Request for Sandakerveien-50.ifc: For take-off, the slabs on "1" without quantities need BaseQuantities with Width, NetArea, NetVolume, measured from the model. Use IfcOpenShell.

First a look at what the model holds.

```python
import ifcopenshell
import ifcopenshell.util.element
import ifcopenshell.util.unit

model = ifcopenshell.open("Sandakerveien-50.ifc")
print(model.schema)
for unit_type in ("LENGTHUNIT", "AREAUNIT", "VOLUMEUNIT"):
    print(unit_type, ifcopenshell.util.unit.calculate_unit_scale(model, unit_type))
storey = next(s for s in model.by_type("IfcBuildingStorey") if s.Name == "1")
slabs = [e for e in ifcopenshell.util.element.get_decomposition(storey) if e.is_a("IfcSlab")]
for e in sorted(slabs, key=lambda e: e.id()):
    print(e.id(), e.is_a(), e.Name, list(ifcopenshell.util.element.get_psets(e, qtos_only=True)), sep=" | ")
```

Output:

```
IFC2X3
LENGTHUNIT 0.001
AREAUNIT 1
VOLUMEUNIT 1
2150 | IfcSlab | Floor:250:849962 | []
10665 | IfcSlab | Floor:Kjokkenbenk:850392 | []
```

```python
import ifcopenshell
import ifcopenshell.api.pset
import ifcopenshell.geom
import ifcopenshell.util.element
import ifcopenshell.util.shape
import ifcopenshell.util.unit

model = ifcopenshell.open("Sandakerveien-50.ifc")
unit_scale = ifcopenshell.util.unit.calculate_unit_scale(model)
area_scale = ifcopenshell.util.unit.calculate_unit_scale(model, "AREAUNIT")
volume_scale = ifcopenshell.util.unit.calculate_unit_scale(model, "VOLUMEUNIT")
settings = ifcopenshell.geom.settings()

storey = next(s for s in model.by_type("IfcBuildingStorey") if s.Name == "1")
slabs = [e for e in ifcopenshell.util.element.get_decomposition(storey) if e.is_a("IfcSlab")]

for e in sorted(slabs, key=lambda e: e.id()):
    if ifcopenshell.util.element.get_psets(e, qtos_only=True, should_inherit=False):
        continue
    # Geometry comes back in metres, in the element's own axes.
    shape = ifcopenshell.geom.create_shape(settings, e)
    values = {
        "Width": ifcopenshell.util.shape.get_z(shape.geometry) / unit_scale,
        "NetArea": ifcopenshell.util.shape.get_footprint_area(shape.geometry) / area_scale,
        "NetVolume": ifcopenshell.util.shape.get_volume(shape.geometry) / volume_scale,
    }
    qto = ifcopenshell.api.pset.add_qto(model, product=e, name="BaseQuantities")
    ifcopenshell.api.pset.edit_qto(model, qto=qto, properties=values)
    print(e.id(), {k: round(v, 3) for k, v in values.items()})

model.write("Sandakerveien-50_updated.ifc")
```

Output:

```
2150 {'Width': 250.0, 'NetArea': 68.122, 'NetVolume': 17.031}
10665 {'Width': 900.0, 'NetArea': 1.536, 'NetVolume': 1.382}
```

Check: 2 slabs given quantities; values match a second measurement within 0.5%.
